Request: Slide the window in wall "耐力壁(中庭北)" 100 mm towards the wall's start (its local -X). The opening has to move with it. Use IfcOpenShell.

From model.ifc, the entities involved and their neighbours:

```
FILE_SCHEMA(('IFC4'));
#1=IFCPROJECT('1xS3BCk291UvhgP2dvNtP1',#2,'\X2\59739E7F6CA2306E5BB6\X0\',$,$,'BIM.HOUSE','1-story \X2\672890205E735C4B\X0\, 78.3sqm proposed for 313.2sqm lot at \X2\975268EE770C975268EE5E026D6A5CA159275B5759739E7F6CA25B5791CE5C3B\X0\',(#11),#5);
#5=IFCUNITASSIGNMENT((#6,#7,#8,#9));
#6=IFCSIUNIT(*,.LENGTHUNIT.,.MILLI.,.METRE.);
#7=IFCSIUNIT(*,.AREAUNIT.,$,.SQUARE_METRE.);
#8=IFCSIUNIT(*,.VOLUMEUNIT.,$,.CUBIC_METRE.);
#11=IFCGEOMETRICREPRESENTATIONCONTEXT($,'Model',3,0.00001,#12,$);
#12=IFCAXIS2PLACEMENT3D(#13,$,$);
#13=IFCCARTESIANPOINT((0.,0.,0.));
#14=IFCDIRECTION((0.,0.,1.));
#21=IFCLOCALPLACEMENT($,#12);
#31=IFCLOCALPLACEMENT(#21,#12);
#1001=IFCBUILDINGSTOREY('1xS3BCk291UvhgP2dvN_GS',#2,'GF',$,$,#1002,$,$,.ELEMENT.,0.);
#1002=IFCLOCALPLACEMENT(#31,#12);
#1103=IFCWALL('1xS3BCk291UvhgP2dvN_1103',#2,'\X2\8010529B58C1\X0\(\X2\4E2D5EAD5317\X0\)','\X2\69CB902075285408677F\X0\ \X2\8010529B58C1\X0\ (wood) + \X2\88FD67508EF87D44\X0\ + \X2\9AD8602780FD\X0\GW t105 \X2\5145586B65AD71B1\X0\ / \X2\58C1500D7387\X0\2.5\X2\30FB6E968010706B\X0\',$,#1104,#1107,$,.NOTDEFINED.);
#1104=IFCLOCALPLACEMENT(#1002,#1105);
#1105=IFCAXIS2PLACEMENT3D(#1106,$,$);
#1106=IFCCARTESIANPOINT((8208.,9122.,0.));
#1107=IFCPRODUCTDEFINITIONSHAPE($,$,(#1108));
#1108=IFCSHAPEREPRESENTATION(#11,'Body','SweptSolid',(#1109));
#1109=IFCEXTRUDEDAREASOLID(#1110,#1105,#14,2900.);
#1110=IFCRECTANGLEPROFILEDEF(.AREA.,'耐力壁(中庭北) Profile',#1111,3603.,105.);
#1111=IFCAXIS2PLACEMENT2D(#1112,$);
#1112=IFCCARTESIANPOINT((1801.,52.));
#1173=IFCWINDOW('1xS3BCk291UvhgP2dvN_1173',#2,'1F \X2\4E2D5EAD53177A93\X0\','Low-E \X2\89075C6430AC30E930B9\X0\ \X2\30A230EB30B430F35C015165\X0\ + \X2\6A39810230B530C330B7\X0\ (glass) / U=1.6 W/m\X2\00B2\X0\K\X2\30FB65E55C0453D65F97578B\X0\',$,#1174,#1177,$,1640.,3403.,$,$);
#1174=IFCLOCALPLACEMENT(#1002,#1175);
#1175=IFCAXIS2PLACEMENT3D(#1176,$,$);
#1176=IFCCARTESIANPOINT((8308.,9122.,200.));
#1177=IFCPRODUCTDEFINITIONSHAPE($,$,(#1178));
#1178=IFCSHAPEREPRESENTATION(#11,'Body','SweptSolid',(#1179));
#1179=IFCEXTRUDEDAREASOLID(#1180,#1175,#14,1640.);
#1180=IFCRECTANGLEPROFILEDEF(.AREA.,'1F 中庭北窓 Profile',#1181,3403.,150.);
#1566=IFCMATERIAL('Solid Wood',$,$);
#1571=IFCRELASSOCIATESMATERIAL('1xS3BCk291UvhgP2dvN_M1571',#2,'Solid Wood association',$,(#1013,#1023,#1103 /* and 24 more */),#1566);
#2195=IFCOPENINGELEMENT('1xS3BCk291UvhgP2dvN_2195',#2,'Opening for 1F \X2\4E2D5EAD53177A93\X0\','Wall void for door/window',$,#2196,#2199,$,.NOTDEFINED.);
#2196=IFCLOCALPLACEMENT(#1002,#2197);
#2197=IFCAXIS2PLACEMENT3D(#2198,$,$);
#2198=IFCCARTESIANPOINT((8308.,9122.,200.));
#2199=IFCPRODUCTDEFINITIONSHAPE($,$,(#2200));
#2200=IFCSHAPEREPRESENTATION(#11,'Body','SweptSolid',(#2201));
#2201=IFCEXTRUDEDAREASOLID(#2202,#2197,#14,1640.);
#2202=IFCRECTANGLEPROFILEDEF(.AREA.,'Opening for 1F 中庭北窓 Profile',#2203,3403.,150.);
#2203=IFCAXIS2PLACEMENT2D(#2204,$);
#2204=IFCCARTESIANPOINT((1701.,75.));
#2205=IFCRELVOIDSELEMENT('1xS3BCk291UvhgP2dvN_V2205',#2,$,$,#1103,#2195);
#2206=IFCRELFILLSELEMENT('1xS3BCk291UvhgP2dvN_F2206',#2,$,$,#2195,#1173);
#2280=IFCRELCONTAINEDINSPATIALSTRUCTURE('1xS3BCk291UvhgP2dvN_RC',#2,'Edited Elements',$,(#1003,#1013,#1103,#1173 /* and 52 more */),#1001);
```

```python
import ifcopenshell
import ifcopenshell.api.geometry
import ifcopenshell.util.placement
import ifcopenshell.util.unit

model = ifcopenshell.open("model.ifc")
unit_scale = ifcopenshell.util.unit.calculate_unit_scale(model)

window = model.by_guid("1xS3BCk291UvhgP2dvN_1173")
opening = window.FillsVoids[0].RelatingOpeningElement
wall = opening.VoidsElements[0].RelatingBuildingElement

wall_matrix = ifcopenshell.util.placement.get_local_placement(wall.ObjectPlacement)
shift = wall_matrix[:3, 0] * -0.1 / unit_scale
before = ifcopenshell.util.placement.get_local_placement(window.ObjectPlacement)[:3, 3].copy()

# The window is not placed relative to its opening, so move both.
for product in (opening, window):
    matrix = ifcopenshell.util.placement.get_local_placement(product.ObjectPlacement)
    matrix[:3, 3] += shift
    ifcopenshell.api.geometry.edit_object_placement(model, product=product, matrix=matrix, is_si=False)

after = ifcopenshell.util.placement.get_local_placement(window.ObjectPlacement)[:3, 3]
print("window moved by", (after - before).round(3) + 0.0)

model.write("model-out.ifc")
```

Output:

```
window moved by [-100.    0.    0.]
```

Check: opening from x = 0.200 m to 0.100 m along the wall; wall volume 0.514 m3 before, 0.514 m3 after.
